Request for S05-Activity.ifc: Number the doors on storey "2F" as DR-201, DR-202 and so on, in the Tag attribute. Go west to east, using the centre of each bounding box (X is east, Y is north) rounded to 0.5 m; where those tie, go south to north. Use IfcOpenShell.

First a look at what the model holds.

```python
import ifcopenshell
import ifcopenshell.util.element
import ifcopenshell.util.placement

model = ifcopenshell.open("S05-Activity.ifc")
print(model.schema)
storey = next(s for s in model.by_type("IfcBuildingStorey") if s.Name == "2F")
doors = [e for e in ifcopenshell.util.element.get_decomposition(storey) if e.is_a("IfcDoor")]
for e in sorted(doors, key=lambda e: e.id()):
    origin = ifcopenshell.util.placement.get_local_placement(e.ObjectPlacement)[:3, 3]
    print(e.id(), e.Tag, e.Name, origin.round(2) + 0.0, sep=" | ")
```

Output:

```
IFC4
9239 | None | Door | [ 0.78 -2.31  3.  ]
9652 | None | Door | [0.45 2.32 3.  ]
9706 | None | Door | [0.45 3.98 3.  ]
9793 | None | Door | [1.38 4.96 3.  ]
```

```python
import ifcopenshell
import ifcopenshell.geom
import ifcopenshell.util.element
import ifcopenshell.util.shape

model = ifcopenshell.open("S05-Activity.ifc")
settings = ifcopenshell.geom.settings()
settings.set("use-world-coords", True)


def centre(element):
    shape = ifcopenshell.geom.create_shape(settings, element)
    return ifcopenshell.util.shape.get_bbox_centroid(shape.geometry)


storey = next(s for s in model.by_type("IfcBuildingStorey") if s.Name == "2F")
doors = [e for e in ifcopenshell.util.element.get_decomposition(storey) if e.is_a("IfcDoor")]

# Insertion points can sit at a corner or the storey origin, so sort by the geometry (in metres).
centres = {e: centre(e) for e in doors}
doors.sort(key=lambda e: (round(centres[e][0] / 0.5), centres[e][1]))

for i, e in enumerate(doors, start=1):
    number = f"DR-2{i:02d}"
    e.Tag = number
    print(e.id(), number)

model.write("S05-Activity_edited.ifc")
```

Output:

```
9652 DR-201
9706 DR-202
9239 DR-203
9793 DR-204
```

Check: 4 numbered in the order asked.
